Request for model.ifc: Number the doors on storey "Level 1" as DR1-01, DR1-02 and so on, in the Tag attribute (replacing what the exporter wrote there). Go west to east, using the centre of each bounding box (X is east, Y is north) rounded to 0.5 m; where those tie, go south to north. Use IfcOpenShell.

First a look at what the model holds.

```python
import ifcopenshell
import ifcopenshell.util.element
import ifcopenshell.util.placement

model = ifcopenshell.open("model.ifc")
print(model.schema)
storey = next(s for s in model.by_type("IfcBuildingStorey") if s.Name == "Level 1")
doors = [e for e in ifcopenshell.util.element.get_decomposition(storey) if e.is_a("IfcDoor")]
for e in sorted(doors, key=lambda e: e.id()):
    origin = ifcopenshell.util.placement.get_local_placement(e.ObjectPlacement)[:3, 3]
    print(e.id(), e.Tag, e.Name, origin.round(2) + 0.0, sep=" | ")
```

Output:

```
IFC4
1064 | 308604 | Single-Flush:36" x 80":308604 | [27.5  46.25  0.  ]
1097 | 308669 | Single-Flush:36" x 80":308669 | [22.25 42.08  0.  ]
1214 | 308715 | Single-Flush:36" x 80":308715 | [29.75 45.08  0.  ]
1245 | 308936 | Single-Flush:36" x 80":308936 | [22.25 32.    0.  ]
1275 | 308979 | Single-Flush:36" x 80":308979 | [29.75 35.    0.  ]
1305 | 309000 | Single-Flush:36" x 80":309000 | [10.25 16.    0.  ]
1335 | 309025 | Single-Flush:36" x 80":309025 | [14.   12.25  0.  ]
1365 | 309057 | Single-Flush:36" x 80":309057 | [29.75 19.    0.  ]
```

```python
import ifcopenshell
import ifcopenshell.geom
import ifcopenshell.util.element
import ifcopenshell.util.shape

model = ifcopenshell.open("model.ifc")
settings = ifcopenshell.geom.settings()
settings.set("use-world-coords", True)


def centre(element):
    shape = ifcopenshell.geom.create_shape(settings, element)
    return ifcopenshell.util.shape.get_bbox_centroid(shape.geometry)


storey = next(s for s in model.by_type("IfcBuildingStorey") if s.Name == "Level 1")
doors = [e for e in ifcopenshell.util.element.get_decomposition(storey) if e.is_a("IfcDoor")]

# Insertion points can sit at a corner or the storey origin, so sort by the geometry (in metres).
centres = {e: centre(e) for e in doors}
doors.sort(key=lambda e: (round(centres[e][0] / 0.5), centres[e][1]))

for i, e in enumerate(doors, start=1):
    number = f"DR1-{i:02d}"
    e.Tag = number
    print(e.id(), number)

model.write("model_updated.ifc")
```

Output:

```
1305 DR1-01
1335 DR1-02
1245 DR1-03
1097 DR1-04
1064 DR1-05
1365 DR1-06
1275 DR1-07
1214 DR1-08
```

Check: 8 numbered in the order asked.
